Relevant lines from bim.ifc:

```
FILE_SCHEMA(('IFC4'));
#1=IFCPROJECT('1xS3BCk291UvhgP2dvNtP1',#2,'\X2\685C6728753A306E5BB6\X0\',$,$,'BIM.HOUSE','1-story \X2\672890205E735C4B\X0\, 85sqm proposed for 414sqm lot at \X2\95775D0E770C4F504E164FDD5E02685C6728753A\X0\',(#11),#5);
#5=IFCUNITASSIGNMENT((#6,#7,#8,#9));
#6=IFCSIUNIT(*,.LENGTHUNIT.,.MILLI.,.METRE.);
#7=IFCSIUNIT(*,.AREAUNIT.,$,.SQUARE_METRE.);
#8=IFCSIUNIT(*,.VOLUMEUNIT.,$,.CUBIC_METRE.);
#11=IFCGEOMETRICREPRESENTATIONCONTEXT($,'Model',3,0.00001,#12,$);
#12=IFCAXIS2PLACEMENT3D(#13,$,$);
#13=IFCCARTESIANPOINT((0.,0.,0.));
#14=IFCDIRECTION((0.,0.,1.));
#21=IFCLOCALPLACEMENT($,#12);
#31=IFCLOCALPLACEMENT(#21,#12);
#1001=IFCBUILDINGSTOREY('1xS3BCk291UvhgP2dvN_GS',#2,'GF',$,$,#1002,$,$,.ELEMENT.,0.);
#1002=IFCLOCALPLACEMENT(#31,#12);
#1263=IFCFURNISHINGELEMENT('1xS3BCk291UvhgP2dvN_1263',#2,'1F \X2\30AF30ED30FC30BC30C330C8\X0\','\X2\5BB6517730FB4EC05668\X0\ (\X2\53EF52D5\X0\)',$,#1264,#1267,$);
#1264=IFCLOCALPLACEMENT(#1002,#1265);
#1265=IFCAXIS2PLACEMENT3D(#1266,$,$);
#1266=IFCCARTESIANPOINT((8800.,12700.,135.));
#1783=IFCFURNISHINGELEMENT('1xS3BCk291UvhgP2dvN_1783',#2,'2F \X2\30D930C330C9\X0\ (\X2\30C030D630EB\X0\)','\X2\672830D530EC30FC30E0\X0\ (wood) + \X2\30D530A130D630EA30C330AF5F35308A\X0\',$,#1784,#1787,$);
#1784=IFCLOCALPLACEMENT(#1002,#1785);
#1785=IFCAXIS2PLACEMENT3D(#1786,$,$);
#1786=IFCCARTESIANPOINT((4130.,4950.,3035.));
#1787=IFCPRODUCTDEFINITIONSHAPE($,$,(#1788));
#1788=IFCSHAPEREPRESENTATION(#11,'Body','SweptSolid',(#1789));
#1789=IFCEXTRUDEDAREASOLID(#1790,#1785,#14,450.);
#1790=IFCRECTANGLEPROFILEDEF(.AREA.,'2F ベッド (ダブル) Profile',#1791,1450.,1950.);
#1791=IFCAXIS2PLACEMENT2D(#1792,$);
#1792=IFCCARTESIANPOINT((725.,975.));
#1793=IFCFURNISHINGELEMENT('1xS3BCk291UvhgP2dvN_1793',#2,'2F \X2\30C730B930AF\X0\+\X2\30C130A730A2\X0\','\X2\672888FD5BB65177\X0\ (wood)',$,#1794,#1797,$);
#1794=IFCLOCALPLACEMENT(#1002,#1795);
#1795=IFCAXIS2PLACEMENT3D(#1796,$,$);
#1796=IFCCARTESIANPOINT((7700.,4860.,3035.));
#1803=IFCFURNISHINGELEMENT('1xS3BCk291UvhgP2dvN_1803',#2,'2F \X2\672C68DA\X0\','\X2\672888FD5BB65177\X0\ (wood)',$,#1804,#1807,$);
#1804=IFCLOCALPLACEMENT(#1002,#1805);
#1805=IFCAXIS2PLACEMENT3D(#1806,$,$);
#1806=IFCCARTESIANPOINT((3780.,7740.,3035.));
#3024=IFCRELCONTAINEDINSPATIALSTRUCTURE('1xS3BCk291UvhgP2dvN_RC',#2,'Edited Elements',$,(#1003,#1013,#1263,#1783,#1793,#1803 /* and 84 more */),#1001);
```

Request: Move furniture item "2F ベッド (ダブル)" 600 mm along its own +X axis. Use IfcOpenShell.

```python
import ifcopenshell
import ifcopenshell.api.geometry
import ifcopenshell.util.placement
import ifcopenshell.util.unit

model = ifcopenshell.open("bim.ifc")
unit_scale = ifcopenshell.util.unit.calculate_unit_scale(model)

item = model.by_guid("1xS3BCk291UvhgP2dvN_1783")
matrix = ifcopenshell.util.placement.get_local_placement(item.ObjectPlacement)
matrix[:3, 3] += matrix[:3, 0] * 0.6 / unit_scale
ifcopenshell.api.geometry.edit_object_placement(model, product=item, matrix=matrix, is_si=False)

print(ifcopenshell.util.placement.get_local_placement(item.ObjectPlacement).round(3) + 0.0)

model.write("bim_v2.ifc")
```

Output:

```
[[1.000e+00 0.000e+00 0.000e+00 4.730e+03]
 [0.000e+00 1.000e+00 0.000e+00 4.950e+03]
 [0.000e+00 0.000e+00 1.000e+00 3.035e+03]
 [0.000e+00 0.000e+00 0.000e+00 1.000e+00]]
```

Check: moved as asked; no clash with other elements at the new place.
